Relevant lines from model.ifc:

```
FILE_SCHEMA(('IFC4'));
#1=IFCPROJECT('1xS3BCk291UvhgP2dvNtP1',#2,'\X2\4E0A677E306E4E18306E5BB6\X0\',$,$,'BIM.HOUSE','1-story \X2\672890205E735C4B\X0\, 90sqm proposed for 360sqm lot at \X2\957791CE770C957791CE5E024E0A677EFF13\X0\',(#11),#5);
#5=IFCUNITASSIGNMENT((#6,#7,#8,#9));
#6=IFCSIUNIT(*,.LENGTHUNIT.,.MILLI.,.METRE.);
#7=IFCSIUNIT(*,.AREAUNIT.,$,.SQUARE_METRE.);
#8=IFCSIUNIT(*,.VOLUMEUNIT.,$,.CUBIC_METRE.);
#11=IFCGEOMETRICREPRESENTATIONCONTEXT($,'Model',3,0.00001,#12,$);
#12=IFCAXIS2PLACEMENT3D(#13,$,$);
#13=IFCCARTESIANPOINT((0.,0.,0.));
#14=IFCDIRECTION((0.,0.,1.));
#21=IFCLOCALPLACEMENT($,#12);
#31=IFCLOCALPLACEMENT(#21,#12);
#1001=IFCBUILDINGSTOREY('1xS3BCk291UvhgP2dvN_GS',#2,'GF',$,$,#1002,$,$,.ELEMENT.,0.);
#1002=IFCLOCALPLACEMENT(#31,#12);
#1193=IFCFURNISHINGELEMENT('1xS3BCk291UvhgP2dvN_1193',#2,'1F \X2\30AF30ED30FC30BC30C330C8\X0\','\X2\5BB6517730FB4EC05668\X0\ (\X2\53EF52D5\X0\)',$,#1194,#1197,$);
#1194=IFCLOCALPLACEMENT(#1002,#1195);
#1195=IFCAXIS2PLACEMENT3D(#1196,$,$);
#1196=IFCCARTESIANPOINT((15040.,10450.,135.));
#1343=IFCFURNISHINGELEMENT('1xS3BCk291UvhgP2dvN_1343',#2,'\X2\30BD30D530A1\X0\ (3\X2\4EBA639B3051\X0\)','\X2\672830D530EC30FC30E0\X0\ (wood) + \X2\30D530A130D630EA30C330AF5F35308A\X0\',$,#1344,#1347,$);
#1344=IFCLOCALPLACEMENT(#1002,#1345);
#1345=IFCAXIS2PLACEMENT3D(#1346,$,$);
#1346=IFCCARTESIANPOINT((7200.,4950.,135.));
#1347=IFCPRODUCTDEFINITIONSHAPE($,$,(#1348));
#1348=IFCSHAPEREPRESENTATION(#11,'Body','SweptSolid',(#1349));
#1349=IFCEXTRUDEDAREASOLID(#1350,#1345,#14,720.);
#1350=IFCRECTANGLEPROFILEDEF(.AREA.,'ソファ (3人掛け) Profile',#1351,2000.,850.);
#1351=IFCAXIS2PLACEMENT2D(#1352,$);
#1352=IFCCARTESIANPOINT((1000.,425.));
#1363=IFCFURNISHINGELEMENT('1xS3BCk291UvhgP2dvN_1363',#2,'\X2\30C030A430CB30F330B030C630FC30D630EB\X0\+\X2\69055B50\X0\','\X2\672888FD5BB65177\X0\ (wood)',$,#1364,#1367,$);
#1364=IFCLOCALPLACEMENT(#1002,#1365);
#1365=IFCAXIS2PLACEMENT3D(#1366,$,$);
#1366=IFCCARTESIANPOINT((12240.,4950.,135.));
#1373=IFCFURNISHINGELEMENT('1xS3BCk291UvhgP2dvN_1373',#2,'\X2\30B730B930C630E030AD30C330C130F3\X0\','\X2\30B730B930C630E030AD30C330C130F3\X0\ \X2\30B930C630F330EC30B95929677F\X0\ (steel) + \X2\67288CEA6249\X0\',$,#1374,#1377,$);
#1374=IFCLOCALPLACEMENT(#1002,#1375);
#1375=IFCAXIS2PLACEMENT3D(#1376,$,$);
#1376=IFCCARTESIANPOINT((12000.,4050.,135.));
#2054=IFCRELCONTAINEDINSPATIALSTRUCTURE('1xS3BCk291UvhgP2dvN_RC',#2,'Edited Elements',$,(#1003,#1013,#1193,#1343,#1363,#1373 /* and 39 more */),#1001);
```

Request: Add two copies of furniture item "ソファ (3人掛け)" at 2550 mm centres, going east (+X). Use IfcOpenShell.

```python
import numpy as np
import ifcopenshell
import ifcopenshell.api.geometry
import ifcopenshell.api.root
import ifcopenshell.util.element
import ifcopenshell.util.placement
import ifcopenshell.util.unit

model = ifcopenshell.open("model.ifc")
unit_scale = ifcopenshell.util.unit.calculate_unit_scale(model)


def reuse_history(source, copy):
    """copy_class also copies each property set's owner history, people and application; keep the originals."""
    for rel in copy.IsDefinedBy:
        if rel.is_a("IfcRelDefinesByProperties") and (history := rel.RelatingPropertyDefinition.OwnerHistory):
            rel.RelatingPropertyDefinition.OwnerHistory = source.OwnerHistory
            ifcopenshell.util.element.remove_deep2(model, history)


source = model.by_guid("1xS3BCk291UvhgP2dvN_1343")
base = ifcopenshell.util.placement.get_local_placement(source.ObjectPlacement)
step = np.array([1.0, 0.0, 0.0]) * 2.55 / unit_scale

for i in range(1, 3):
    copy = ifcopenshell.api.root.copy_class(model, product=source)
    copy.Representation = ifcopenshell.util.element.copy_deep(
        model, source.Representation, exclude=["IfcGeometricRepresentationContext", "IfcRepresentationMap"]
    )
    reuse_history(source, copy)
    matrix = base.copy()
    matrix[:3, 3] += i * step
    print("added at", matrix[:3, 3].round(3) + 0.0)
    ifcopenshell.api.geometry.edit_object_placement(model, product=copy, matrix=matrix, is_si=False)

model.write("model_v2.ifc")
```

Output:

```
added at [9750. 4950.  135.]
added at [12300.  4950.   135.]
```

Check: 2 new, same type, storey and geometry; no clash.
